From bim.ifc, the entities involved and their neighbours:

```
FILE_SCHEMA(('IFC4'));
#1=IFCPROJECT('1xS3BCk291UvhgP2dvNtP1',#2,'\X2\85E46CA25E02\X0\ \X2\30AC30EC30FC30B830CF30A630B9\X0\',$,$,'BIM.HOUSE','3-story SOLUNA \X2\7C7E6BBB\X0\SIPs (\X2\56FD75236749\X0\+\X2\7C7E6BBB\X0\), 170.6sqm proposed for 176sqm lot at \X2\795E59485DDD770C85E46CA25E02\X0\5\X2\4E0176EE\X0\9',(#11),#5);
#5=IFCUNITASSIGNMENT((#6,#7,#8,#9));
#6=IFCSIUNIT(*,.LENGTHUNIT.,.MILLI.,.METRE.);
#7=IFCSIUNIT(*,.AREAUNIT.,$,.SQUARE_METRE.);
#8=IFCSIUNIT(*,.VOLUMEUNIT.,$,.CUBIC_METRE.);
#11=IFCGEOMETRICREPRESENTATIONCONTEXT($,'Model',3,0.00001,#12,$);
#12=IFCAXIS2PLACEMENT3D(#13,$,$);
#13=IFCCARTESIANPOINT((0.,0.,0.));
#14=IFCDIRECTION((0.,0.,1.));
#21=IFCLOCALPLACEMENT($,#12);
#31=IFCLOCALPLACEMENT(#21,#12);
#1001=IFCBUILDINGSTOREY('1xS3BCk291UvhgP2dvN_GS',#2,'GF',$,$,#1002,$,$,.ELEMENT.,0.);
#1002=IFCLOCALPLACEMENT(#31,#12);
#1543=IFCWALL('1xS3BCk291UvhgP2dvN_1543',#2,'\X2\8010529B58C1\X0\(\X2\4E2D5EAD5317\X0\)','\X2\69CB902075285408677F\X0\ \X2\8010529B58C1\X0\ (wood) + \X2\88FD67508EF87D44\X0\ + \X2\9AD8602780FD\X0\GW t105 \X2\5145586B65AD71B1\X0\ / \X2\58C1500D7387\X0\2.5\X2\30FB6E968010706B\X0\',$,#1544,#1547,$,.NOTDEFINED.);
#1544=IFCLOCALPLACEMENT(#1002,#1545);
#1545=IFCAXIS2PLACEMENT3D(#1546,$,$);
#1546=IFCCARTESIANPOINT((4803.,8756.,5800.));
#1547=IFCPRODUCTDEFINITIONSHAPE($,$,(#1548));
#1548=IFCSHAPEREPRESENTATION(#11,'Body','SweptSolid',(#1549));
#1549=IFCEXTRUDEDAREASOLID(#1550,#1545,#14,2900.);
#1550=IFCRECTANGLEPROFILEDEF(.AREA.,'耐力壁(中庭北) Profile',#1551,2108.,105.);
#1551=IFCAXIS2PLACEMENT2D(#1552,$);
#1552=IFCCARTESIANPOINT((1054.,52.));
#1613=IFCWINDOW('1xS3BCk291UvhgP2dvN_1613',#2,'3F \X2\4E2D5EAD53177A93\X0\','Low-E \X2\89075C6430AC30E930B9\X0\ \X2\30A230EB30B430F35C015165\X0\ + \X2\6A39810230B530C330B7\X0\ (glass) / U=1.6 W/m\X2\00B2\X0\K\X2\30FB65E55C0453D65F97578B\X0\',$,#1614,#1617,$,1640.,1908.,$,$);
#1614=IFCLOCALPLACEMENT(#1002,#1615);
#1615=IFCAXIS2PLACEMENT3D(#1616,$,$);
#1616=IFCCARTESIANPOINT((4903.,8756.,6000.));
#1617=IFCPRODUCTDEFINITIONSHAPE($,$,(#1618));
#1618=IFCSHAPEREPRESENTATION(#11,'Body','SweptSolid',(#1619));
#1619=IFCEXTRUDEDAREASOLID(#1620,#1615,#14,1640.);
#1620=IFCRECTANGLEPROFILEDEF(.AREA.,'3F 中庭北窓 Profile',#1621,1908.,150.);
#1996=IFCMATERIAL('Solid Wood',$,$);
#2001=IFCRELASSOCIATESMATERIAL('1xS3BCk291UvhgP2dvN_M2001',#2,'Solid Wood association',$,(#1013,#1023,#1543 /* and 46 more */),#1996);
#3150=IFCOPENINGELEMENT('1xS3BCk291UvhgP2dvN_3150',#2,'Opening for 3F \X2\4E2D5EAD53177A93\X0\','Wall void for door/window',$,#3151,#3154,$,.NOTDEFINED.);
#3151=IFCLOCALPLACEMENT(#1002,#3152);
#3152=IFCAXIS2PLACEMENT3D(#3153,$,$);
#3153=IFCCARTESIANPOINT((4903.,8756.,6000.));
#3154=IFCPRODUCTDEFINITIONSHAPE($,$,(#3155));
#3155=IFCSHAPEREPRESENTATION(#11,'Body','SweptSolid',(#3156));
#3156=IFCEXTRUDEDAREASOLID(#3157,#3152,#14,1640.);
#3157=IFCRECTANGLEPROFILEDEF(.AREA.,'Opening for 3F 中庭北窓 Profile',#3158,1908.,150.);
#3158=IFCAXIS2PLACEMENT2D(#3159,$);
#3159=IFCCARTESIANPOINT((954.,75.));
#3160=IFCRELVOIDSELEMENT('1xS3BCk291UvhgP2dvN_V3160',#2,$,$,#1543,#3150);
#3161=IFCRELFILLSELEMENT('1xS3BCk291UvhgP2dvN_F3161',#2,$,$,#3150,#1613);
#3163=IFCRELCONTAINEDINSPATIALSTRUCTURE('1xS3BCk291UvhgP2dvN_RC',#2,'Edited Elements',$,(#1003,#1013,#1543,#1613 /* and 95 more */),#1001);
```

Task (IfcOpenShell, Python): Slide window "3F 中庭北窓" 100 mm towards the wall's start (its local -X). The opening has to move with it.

```python
import ifcopenshell
import ifcopenshell.api.geometry
import ifcopenshell.util.placement
import ifcopenshell.util.unit

model = ifcopenshell.open("bim.ifc")
unit_scale = ifcopenshell.util.unit.calculate_unit_scale(model)

window = model.by_id(1613)
opening = window.FillsVoids[0].RelatingOpeningElement
wall = opening.VoidsElements[0].RelatingBuildingElement

wall_matrix = ifcopenshell.util.placement.get_local_placement(wall.ObjectPlacement)
shift = wall_matrix[:3, 0] * -0.1 / unit_scale
before = ifcopenshell.util.placement.get_local_placement(window.ObjectPlacement)[:3, 3].copy()

# The window is not placed relative to its opening, so move both.
for product in (opening, window):
    matrix = ifcopenshell.util.placement.get_local_placement(product.ObjectPlacement)
    matrix[:3, 3] += shift
    ifcopenshell.api.geometry.edit_object_placement(model, product=product, matrix=matrix, is_si=False)

after = ifcopenshell.util.placement.get_local_placement(window.ObjectPlacement)[:3, 3]
print("window moved by", (after - before).round(3) + 0.0)

model.write("bim_v2.ifc")
```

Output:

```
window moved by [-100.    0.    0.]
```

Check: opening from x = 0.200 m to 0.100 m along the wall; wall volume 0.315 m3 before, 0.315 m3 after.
